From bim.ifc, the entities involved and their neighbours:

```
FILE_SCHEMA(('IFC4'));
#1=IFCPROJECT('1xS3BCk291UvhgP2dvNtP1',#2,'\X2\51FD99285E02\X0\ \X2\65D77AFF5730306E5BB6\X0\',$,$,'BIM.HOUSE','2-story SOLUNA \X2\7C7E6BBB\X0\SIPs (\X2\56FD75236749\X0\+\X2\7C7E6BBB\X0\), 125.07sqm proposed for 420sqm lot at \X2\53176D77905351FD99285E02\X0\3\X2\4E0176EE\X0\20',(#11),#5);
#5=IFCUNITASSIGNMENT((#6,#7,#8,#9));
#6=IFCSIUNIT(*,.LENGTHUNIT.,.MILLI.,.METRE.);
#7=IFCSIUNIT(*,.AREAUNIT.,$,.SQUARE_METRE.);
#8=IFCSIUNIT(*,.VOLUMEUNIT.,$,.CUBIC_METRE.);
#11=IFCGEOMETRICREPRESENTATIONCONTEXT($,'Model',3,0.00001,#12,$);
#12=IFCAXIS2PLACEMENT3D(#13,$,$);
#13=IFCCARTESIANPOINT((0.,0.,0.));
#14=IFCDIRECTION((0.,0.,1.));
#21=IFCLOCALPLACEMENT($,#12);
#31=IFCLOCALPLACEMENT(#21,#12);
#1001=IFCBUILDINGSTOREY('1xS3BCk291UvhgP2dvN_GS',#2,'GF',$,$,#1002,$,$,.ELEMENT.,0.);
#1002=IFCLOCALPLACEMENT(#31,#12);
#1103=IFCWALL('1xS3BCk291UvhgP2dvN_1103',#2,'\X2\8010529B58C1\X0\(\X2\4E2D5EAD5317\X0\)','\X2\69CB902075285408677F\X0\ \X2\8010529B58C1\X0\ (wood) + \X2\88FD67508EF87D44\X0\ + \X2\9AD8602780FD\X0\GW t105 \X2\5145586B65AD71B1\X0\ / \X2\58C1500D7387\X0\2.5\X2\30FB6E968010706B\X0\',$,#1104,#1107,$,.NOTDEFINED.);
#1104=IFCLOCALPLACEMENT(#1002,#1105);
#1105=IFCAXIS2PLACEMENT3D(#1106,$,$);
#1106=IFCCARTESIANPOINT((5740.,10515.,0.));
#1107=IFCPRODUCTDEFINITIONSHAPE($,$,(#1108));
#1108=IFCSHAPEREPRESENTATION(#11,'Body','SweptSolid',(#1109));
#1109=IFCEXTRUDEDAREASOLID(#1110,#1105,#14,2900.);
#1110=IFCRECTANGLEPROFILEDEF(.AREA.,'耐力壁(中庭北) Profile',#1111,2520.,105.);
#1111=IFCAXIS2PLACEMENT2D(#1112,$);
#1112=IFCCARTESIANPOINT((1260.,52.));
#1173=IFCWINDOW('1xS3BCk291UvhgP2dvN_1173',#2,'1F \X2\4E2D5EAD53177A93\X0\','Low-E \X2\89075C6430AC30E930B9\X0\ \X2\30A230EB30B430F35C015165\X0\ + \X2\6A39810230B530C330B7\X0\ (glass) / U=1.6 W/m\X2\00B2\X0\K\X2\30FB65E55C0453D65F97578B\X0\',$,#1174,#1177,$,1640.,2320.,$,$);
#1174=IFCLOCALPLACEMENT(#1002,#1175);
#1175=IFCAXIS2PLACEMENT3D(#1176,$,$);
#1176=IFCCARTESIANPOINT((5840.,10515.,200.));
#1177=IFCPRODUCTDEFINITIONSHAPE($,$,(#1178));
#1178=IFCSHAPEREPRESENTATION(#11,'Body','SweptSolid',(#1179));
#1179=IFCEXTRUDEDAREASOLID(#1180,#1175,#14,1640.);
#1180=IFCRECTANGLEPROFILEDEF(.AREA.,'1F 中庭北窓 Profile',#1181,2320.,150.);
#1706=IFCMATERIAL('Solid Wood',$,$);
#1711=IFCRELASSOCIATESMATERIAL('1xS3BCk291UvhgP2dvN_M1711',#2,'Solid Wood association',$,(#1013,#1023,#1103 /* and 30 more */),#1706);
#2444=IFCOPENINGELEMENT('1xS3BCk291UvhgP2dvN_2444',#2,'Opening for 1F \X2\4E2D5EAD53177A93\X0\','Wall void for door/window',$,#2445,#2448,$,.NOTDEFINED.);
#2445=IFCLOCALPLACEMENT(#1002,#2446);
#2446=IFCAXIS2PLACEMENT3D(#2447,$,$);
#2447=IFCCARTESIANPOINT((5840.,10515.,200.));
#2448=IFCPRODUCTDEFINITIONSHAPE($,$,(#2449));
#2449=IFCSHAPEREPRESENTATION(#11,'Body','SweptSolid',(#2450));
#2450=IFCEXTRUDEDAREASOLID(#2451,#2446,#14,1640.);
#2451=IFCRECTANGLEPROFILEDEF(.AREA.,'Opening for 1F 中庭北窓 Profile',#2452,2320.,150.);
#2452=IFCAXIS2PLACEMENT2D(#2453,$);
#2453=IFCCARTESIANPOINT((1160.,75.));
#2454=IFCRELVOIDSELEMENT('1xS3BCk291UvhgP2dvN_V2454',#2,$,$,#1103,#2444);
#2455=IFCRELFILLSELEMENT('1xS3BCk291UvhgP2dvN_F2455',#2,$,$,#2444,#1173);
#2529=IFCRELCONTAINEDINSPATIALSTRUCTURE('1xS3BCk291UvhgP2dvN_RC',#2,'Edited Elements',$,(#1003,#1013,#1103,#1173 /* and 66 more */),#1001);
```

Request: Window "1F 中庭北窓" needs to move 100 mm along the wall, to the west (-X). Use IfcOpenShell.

```python
import ifcopenshell
import ifcopenshell.api.geometry
import ifcopenshell.util.placement
import ifcopenshell.util.unit

model = ifcopenshell.open("bim.ifc")
unit_scale = ifcopenshell.util.unit.calculate_unit_scale(model)

window = model.by_guid("1xS3BCk291UvhgP2dvN_1173")
opening = window.FillsVoids[0].RelatingOpeningElement
wall = opening.VoidsElements[0].RelatingBuildingElement

wall_matrix = ifcopenshell.util.placement.get_local_placement(wall.ObjectPlacement)
shift = wall_matrix[:3, 0] * -0.1 / unit_scale
before = ifcopenshell.util.placement.get_local_placement(window.ObjectPlacement)[:3, 3].copy()

# The window is not placed relative to its opening, so move both.
for product in (opening, window):
    matrix = ifcopenshell.util.placement.get_local_placement(product.ObjectPlacement)
    matrix[:3, 3] += shift
    ifcopenshell.api.geometry.edit_object_placement(model, product=product, matrix=matrix, is_si=False)

after = ifcopenshell.util.placement.get_local_placement(window.ObjectPlacement)[:3, 3]
print("window moved by", (after - before).round(3) + 0.0)

model.write("bim_v2.ifc")
```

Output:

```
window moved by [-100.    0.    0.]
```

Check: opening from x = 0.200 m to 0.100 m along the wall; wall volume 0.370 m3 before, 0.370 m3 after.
